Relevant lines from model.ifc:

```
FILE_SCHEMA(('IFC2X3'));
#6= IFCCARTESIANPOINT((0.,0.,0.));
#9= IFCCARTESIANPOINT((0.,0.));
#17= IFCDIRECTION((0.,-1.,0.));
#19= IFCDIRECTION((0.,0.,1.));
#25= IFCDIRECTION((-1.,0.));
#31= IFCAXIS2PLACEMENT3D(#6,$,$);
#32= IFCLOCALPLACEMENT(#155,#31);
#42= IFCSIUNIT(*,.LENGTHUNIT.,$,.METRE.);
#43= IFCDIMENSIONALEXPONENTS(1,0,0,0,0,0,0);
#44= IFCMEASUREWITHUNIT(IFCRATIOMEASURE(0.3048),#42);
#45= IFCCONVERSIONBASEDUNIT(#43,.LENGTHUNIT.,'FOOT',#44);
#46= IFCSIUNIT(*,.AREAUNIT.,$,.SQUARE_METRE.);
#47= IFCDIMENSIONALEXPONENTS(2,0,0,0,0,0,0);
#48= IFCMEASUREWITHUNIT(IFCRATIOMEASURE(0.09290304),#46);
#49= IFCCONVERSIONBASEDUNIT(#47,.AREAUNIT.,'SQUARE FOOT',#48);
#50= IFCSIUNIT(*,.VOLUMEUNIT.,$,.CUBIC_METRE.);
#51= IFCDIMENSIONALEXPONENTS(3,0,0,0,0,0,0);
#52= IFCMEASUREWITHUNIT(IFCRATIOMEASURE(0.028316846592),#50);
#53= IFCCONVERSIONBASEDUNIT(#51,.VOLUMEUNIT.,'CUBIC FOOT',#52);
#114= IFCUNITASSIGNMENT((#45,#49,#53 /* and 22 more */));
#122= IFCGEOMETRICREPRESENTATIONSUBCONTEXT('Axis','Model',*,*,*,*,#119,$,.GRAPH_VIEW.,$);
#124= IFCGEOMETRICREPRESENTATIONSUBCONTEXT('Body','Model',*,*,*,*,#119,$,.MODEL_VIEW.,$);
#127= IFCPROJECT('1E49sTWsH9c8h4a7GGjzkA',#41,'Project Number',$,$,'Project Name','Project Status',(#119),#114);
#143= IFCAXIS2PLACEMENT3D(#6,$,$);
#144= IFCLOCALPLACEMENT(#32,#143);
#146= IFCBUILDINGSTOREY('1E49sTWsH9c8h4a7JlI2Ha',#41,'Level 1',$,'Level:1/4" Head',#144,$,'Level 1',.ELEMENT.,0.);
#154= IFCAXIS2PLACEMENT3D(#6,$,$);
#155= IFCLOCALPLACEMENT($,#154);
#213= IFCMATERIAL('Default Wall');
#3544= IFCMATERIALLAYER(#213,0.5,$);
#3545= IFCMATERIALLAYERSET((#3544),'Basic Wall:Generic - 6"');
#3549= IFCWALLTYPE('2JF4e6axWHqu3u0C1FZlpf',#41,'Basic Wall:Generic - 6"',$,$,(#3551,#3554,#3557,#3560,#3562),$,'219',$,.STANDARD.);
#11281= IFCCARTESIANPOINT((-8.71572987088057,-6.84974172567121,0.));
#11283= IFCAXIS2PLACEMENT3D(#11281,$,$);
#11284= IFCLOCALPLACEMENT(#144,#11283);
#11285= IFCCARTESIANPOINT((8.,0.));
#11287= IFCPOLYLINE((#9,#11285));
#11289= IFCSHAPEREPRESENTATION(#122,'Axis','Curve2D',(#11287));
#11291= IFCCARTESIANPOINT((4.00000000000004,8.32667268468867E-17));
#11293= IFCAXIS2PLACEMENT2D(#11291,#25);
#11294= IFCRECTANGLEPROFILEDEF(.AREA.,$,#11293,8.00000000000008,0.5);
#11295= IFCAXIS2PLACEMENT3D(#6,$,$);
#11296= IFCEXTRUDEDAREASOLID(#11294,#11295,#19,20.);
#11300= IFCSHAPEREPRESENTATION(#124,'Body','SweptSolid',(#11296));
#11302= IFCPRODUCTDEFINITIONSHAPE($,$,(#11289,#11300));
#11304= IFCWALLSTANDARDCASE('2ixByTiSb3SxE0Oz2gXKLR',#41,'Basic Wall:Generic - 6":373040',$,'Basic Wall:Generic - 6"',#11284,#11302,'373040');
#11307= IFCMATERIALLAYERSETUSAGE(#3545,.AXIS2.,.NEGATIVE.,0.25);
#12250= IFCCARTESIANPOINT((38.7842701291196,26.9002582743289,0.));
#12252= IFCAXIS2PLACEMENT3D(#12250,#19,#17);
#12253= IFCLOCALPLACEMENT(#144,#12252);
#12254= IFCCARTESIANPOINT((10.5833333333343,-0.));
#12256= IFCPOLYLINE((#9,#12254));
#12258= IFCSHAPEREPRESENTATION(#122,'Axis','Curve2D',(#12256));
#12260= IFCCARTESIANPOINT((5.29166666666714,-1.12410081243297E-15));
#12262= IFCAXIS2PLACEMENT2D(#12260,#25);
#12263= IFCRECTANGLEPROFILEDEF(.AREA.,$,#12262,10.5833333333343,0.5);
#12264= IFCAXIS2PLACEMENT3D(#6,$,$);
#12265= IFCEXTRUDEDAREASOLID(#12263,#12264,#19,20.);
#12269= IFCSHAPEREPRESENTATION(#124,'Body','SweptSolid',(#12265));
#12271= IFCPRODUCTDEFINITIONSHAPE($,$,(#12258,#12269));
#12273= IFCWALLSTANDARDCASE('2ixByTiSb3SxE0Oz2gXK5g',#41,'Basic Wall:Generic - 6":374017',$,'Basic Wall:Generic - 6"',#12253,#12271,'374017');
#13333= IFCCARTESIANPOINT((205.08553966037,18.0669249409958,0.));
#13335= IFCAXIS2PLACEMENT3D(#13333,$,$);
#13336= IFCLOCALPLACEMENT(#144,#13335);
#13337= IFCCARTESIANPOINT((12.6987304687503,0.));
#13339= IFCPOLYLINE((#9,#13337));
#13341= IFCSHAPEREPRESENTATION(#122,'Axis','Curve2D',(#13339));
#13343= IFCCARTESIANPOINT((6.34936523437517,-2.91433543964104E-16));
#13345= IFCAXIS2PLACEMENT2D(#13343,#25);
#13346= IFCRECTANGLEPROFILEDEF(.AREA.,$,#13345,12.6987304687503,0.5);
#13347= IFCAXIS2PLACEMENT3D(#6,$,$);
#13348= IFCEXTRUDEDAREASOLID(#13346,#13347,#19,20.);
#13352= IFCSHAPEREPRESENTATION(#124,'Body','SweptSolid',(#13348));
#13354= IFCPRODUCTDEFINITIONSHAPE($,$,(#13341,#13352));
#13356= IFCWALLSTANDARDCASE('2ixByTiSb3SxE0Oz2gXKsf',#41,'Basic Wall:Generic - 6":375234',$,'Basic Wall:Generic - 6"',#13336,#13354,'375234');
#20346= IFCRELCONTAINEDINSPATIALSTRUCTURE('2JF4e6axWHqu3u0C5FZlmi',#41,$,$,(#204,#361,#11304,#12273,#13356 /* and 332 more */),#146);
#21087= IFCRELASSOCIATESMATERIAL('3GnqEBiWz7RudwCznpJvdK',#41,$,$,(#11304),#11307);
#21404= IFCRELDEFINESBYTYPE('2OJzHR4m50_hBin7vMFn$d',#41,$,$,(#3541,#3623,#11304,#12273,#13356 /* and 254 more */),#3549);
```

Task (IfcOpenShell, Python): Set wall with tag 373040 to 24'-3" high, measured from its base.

```python
import ifcopenshell
import ifcopenshell.geom
import ifcopenshell.util.representation
import ifcopenshell.util.shape
import ifcopenshell.util.unit

model = ifcopenshell.open("model.ifc")
unit_scale = ifcopenshell.util.unit.calculate_unit_scale(model)
settings = ifcopenshell.geom.settings()


def volume(element):
    """Net volume in cubic metres, openings subtracted."""
    shape = ifcopenshell.geom.create_shape(settings, element)
    return ifcopenshell.util.shape.get_volume(shape.geometry)


wall = model.by_guid("2ixByTiSb3SxE0Oz2gXKLR")
before = volume(wall)

body = ifcopenshell.util.representation.get_representation(wall, "Model", "Body")
solid = body.Items[0]
old_height = solid.Depth
solid.Depth = 291 * 0.0254 / unit_scale
after = volume(wall)

print(f"height {old_height:g} -> {solid.Depth:g}, volume {before:.3f} -> {after:.3f} m3")

model.write("model_updated.ifc")
```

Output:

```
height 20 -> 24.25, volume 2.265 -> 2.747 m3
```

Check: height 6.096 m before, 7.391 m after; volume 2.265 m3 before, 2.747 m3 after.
